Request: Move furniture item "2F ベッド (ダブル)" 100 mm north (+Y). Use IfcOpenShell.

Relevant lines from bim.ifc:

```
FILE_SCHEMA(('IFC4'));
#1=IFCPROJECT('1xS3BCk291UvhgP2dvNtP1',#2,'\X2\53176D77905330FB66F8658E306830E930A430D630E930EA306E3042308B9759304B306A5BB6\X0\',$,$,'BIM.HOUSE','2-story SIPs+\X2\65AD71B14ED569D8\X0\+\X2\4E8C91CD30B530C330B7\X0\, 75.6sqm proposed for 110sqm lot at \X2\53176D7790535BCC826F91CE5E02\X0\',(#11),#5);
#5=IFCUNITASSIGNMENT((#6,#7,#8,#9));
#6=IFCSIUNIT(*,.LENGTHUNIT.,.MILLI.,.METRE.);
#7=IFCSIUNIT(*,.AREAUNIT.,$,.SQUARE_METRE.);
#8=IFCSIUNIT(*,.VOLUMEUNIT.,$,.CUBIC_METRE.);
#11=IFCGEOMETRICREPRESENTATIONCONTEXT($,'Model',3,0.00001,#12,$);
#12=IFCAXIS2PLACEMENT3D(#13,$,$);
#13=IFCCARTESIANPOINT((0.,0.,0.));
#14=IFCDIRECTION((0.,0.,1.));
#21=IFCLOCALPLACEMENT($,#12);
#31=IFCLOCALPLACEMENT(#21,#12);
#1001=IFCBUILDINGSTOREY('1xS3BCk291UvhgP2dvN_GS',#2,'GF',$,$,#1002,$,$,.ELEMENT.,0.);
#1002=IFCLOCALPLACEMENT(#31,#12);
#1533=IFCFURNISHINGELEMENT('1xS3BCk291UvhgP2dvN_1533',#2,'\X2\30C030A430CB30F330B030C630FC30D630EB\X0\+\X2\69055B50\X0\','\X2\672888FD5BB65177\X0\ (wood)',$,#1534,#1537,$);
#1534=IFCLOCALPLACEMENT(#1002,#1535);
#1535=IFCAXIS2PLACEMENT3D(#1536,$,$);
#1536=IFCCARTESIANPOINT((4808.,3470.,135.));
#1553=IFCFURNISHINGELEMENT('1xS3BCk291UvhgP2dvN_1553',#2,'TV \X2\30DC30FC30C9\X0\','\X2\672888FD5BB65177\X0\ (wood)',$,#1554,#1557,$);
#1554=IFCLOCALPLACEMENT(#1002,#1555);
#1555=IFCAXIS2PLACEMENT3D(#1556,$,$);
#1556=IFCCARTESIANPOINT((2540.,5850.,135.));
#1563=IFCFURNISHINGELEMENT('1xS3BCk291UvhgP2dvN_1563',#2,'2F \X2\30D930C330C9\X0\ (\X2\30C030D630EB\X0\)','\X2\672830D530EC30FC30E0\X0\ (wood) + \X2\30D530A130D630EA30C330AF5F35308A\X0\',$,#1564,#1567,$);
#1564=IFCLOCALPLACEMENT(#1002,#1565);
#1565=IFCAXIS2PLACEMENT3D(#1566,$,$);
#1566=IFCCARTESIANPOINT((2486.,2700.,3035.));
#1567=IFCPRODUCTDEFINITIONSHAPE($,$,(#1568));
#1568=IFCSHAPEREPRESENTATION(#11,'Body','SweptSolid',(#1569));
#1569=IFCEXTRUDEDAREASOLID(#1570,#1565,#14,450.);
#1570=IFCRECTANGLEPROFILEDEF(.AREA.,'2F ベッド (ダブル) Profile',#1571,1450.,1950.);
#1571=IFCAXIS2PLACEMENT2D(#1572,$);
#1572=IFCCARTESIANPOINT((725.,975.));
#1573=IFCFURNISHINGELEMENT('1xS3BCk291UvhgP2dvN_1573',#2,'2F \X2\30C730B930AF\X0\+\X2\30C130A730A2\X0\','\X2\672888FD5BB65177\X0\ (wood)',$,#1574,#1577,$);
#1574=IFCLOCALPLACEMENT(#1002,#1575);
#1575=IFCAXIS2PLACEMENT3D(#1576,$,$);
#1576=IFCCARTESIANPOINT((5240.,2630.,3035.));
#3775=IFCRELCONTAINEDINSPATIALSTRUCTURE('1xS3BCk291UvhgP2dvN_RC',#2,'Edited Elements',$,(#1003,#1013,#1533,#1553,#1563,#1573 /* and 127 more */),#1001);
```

```python
import ifcopenshell
import ifcopenshell.api.geometry
import ifcopenshell.util.placement
import ifcopenshell.util.unit

model = ifcopenshell.open("bim.ifc")
unit_scale = ifcopenshell.util.unit.calculate_unit_scale(model)

item = model.by_guid("1xS3BCk291UvhgP2dvN_1563")
matrix = ifcopenshell.util.placement.get_local_placement(item.ObjectPlacement)
matrix[1, 3] += 0.1 / unit_scale
ifcopenshell.api.geometry.edit_object_placement(model, product=item, matrix=matrix, is_si=False)

print(ifcopenshell.util.placement.get_local_placement(item.ObjectPlacement).round(3) + 0.0)

model.write("bim_v2.ifc")
```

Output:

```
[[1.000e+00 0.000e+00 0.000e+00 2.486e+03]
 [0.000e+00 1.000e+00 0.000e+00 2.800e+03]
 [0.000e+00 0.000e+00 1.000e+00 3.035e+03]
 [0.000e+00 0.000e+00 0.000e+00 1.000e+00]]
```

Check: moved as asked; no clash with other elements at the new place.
